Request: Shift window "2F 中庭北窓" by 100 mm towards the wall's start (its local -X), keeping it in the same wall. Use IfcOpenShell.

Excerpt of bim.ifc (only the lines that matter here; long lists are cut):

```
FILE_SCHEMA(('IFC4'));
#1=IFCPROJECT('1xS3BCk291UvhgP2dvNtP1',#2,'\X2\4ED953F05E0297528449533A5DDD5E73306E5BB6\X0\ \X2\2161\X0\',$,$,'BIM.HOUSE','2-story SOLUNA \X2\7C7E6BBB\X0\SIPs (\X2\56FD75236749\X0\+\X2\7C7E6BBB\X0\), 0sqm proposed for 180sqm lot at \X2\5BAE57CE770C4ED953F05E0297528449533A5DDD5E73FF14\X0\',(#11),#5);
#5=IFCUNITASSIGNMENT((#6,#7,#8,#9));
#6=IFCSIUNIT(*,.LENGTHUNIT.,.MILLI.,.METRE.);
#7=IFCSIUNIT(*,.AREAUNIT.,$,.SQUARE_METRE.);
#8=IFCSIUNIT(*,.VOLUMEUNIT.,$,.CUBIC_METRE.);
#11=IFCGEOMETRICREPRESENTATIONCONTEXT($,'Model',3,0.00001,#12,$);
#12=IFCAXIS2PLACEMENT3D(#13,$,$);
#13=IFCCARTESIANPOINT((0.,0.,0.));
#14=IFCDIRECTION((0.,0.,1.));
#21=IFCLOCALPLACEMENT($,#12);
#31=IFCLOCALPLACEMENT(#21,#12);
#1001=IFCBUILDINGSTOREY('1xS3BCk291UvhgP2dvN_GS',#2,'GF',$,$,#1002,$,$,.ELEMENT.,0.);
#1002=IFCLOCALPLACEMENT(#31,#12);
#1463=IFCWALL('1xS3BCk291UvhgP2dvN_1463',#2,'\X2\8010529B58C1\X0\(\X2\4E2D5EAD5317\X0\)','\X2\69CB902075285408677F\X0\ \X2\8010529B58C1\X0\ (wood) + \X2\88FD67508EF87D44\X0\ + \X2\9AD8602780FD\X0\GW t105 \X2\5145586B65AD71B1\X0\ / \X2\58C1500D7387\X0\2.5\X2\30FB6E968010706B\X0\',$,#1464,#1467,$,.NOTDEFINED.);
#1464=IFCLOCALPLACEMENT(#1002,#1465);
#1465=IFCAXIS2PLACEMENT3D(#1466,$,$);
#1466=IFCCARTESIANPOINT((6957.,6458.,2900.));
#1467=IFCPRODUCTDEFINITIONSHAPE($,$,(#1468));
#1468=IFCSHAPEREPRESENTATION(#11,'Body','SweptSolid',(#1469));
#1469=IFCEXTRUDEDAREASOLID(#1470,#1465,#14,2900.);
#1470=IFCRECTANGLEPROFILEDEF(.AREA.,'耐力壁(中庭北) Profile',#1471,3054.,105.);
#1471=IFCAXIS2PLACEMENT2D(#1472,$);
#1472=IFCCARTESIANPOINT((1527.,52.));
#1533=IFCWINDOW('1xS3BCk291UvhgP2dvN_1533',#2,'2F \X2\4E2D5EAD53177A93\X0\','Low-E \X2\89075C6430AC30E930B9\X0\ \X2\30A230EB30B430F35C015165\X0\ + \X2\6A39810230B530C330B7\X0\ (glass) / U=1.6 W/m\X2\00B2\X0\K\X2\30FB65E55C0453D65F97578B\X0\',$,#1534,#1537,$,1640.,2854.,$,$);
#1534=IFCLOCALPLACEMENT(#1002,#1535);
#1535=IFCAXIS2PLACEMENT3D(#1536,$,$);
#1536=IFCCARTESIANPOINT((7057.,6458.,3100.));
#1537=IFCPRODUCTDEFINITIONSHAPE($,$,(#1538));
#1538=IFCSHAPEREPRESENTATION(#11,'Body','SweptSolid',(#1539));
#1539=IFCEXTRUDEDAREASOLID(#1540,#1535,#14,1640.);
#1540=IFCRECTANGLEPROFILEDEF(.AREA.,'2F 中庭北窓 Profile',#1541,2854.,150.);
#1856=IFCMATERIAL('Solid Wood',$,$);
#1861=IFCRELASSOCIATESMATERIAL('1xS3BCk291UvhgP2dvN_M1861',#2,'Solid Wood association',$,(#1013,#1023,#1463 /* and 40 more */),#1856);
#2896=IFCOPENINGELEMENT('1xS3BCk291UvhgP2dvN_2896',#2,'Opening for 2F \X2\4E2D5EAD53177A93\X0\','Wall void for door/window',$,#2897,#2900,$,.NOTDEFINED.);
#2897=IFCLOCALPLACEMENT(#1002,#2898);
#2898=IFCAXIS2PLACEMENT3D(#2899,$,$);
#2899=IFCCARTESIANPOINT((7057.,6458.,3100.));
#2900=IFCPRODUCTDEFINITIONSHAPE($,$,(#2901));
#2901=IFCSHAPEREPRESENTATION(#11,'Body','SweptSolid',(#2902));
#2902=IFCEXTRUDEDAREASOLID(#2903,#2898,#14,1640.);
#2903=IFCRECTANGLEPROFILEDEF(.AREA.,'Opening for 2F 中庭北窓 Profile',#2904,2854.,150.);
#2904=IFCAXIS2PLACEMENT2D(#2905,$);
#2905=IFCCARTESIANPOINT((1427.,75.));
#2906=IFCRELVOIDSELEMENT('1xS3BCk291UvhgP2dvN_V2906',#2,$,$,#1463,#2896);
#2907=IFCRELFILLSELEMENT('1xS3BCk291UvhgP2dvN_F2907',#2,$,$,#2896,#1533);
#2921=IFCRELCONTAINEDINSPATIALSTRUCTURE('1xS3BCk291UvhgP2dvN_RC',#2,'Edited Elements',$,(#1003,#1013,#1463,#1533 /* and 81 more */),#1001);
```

```python
import ifcopenshell
import ifcopenshell.api.geometry
import ifcopenshell.util.placement

model = ifcopenshell.open("bim.ifc")

window = model.by_guid("1xS3BCk291UvhgP2dvN_1533")
opening = window.FillsVoids[0].RelatingOpeningElement
wall = opening.VoidsElements[0].RelatingBuildingElement

wall_matrix = ifcopenshell.util.placement.get_local_placement(wall.ObjectPlacement)
shift = wall_matrix[:3, 0] * -100.0
before = ifcopenshell.util.placement.get_local_placement(window.ObjectPlacement)[:3, 3].copy()

# The window is not placed relative to its opening, so move both.
for product in (opening, window):
    matrix = ifcopenshell.util.placement.get_local_placement(product.ObjectPlacement)
    matrix[:3, 3] += shift
    ifcopenshell.api.geometry.edit_object_placement(model, product=product, matrix=matrix, is_si=False)

after = ifcopenshell.util.placement.get_local_placement(window.ObjectPlacement)[:3, 3]
print("window moved by", (after - before).round(3) + 0.0)

model.write("bim_edited.ifc")
```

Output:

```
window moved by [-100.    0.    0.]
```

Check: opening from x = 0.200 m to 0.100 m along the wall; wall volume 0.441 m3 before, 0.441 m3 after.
